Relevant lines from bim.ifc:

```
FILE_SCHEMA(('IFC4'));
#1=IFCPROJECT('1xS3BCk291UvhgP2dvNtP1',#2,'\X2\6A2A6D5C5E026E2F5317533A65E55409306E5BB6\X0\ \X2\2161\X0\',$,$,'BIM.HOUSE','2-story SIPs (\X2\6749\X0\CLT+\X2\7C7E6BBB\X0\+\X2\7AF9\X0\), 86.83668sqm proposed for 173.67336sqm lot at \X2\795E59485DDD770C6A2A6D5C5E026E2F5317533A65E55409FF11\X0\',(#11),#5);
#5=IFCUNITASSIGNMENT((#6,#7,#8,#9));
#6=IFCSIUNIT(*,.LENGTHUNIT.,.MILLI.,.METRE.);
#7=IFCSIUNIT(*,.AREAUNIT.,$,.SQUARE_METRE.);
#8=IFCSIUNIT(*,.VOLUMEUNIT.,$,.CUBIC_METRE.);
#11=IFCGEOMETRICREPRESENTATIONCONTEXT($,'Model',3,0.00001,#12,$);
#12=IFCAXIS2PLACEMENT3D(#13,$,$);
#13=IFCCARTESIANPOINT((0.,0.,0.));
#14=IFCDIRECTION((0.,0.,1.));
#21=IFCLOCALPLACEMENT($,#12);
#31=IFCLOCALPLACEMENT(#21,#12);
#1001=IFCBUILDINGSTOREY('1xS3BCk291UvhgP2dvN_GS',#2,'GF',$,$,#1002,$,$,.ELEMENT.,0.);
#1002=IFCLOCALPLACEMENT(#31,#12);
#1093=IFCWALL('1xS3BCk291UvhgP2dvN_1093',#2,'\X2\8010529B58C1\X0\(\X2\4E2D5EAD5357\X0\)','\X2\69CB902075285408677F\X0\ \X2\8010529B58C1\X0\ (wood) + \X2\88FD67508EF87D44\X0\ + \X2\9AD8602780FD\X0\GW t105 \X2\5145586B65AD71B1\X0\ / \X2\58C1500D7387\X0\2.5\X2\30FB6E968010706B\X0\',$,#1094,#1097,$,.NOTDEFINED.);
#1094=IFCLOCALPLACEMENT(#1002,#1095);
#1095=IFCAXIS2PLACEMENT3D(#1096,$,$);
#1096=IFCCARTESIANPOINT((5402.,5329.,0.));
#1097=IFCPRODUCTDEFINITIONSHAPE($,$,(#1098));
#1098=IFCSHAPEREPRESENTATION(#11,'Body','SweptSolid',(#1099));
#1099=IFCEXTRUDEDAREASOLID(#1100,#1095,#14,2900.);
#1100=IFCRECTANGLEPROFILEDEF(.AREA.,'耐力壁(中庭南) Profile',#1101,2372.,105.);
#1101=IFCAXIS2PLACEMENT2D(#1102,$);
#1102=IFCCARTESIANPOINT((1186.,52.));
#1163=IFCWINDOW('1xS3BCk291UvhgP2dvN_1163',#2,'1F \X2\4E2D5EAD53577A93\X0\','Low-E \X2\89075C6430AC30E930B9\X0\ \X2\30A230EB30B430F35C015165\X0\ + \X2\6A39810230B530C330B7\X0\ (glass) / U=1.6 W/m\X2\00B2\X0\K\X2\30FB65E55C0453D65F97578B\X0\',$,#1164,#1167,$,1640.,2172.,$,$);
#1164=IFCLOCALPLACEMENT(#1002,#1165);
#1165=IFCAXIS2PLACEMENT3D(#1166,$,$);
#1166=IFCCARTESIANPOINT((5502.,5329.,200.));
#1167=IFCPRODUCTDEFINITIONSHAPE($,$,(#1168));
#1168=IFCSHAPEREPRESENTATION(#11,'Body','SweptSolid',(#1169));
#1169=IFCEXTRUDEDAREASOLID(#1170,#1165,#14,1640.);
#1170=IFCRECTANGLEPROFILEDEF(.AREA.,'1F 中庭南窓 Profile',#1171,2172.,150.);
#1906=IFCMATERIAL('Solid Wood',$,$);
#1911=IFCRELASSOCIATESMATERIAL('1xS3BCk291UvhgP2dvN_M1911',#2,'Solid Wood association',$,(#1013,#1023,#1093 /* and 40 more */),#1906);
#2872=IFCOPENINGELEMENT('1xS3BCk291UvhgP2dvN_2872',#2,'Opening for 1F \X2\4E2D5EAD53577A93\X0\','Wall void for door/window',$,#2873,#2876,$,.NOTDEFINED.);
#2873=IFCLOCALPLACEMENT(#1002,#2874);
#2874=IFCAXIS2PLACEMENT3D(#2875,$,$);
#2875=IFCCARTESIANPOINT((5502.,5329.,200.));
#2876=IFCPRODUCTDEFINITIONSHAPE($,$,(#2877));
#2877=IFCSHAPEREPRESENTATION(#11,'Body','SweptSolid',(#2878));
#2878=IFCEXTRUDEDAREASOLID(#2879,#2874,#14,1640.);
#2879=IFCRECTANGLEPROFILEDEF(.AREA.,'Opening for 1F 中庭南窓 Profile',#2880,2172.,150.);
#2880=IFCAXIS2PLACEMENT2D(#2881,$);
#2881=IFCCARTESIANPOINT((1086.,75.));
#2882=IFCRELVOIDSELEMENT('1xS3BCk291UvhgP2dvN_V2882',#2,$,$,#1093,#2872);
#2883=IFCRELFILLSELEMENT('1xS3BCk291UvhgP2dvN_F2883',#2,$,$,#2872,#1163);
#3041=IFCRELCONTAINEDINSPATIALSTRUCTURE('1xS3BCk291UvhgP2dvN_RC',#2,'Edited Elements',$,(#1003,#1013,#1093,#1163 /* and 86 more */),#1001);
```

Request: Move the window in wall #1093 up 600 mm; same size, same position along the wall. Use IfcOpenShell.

```python
import numpy as np
import ifcopenshell
import ifcopenshell.api.geometry
import ifcopenshell.util.placement
import ifcopenshell.util.unit

model = ifcopenshell.open("bim.ifc")
unit_scale = ifcopenshell.util.unit.calculate_unit_scale(model)

window = model.by_guid("1xS3BCk291UvhgP2dvN_1163")
opening = window.FillsVoids[0].RelatingOpeningElement
dz = 600.0

shift = np.array([0.0, 0.0, dz])
# The window is not placed relative to its opening, so move both.
for product in (opening, window):
    matrix = ifcopenshell.util.placement.get_local_placement(product.ObjectPlacement)
    matrix[:3, 3] += shift
    ifcopenshell.api.geometry.edit_object_placement(model, product=product, matrix=matrix, is_si=False)

print(f"moved by {dz * unit_scale:+.3f} m")

model.write("bim-out.ifc")
```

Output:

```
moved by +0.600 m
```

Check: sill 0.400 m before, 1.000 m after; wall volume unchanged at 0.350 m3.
